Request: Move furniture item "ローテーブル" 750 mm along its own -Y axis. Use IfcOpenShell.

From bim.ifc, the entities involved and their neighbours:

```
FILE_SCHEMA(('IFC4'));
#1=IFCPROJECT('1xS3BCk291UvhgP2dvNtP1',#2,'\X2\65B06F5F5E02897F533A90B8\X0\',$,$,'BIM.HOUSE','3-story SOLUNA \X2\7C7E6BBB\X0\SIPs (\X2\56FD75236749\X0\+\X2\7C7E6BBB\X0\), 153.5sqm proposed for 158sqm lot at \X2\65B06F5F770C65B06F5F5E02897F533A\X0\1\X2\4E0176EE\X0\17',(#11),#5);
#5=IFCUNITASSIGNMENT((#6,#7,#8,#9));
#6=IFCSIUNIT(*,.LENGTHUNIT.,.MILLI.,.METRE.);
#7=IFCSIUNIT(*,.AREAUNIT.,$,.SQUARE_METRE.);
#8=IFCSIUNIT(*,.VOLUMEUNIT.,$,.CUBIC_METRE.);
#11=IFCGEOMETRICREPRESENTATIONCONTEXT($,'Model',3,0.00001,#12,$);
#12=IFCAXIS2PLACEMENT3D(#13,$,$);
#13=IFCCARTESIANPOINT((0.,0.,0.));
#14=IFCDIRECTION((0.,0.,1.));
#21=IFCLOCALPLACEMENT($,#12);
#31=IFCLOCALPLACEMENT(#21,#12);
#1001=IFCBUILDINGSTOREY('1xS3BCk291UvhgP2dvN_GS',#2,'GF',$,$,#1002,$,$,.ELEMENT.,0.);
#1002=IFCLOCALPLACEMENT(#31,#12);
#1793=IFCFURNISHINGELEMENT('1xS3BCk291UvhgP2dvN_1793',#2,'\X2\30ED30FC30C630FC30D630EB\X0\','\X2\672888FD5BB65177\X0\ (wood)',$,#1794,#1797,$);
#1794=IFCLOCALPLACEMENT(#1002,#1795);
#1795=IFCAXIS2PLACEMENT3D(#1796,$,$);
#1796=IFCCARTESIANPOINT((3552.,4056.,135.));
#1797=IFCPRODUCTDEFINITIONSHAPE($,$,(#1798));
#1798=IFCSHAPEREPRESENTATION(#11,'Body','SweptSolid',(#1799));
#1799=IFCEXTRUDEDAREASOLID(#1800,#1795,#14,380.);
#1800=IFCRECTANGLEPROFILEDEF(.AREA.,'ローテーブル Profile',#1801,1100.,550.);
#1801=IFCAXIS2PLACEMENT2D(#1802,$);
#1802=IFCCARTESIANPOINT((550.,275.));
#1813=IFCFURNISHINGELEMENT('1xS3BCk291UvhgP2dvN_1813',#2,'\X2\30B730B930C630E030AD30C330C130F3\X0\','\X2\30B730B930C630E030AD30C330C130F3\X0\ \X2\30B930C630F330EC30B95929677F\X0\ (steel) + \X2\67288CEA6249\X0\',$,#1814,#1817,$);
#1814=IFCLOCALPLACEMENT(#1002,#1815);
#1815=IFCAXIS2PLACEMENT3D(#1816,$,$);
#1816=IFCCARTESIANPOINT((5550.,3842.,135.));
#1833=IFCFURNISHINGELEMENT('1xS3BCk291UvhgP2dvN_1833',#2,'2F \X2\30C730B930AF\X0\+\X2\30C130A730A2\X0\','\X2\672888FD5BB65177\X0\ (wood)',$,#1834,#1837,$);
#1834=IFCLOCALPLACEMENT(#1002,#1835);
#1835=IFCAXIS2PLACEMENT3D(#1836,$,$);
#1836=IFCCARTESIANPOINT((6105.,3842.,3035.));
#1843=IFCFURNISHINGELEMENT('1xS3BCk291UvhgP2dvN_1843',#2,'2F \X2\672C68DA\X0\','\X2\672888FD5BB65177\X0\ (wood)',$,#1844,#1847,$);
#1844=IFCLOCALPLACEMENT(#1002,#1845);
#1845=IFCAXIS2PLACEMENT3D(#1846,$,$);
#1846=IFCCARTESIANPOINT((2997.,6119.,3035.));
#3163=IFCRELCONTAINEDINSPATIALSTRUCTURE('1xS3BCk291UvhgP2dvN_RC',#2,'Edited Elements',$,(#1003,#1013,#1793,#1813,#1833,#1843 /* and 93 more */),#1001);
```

```python
import ifcopenshell
import ifcopenshell.api.geometry
import ifcopenshell.util.placement
import ifcopenshell.util.unit

model = ifcopenshell.open("bim.ifc")
unit_scale = ifcopenshell.util.unit.calculate_unit_scale(model)

item = model.by_guid("1xS3BCk291UvhgP2dvN_1793")
matrix = ifcopenshell.util.placement.get_local_placement(item.ObjectPlacement)
matrix[:3, 3] -= matrix[:3, 1] * 0.75 / unit_scale
ifcopenshell.api.geometry.edit_object_placement(model, product=item, matrix=matrix, is_si=False)

print(ifcopenshell.util.placement.get_local_placement(item.ObjectPlacement).round(3) + 0.0)

model.write("bim_updated.ifc")
```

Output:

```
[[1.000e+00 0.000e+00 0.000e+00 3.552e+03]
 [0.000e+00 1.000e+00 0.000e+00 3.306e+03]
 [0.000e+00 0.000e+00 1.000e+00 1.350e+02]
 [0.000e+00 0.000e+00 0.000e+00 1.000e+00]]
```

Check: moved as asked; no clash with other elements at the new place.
